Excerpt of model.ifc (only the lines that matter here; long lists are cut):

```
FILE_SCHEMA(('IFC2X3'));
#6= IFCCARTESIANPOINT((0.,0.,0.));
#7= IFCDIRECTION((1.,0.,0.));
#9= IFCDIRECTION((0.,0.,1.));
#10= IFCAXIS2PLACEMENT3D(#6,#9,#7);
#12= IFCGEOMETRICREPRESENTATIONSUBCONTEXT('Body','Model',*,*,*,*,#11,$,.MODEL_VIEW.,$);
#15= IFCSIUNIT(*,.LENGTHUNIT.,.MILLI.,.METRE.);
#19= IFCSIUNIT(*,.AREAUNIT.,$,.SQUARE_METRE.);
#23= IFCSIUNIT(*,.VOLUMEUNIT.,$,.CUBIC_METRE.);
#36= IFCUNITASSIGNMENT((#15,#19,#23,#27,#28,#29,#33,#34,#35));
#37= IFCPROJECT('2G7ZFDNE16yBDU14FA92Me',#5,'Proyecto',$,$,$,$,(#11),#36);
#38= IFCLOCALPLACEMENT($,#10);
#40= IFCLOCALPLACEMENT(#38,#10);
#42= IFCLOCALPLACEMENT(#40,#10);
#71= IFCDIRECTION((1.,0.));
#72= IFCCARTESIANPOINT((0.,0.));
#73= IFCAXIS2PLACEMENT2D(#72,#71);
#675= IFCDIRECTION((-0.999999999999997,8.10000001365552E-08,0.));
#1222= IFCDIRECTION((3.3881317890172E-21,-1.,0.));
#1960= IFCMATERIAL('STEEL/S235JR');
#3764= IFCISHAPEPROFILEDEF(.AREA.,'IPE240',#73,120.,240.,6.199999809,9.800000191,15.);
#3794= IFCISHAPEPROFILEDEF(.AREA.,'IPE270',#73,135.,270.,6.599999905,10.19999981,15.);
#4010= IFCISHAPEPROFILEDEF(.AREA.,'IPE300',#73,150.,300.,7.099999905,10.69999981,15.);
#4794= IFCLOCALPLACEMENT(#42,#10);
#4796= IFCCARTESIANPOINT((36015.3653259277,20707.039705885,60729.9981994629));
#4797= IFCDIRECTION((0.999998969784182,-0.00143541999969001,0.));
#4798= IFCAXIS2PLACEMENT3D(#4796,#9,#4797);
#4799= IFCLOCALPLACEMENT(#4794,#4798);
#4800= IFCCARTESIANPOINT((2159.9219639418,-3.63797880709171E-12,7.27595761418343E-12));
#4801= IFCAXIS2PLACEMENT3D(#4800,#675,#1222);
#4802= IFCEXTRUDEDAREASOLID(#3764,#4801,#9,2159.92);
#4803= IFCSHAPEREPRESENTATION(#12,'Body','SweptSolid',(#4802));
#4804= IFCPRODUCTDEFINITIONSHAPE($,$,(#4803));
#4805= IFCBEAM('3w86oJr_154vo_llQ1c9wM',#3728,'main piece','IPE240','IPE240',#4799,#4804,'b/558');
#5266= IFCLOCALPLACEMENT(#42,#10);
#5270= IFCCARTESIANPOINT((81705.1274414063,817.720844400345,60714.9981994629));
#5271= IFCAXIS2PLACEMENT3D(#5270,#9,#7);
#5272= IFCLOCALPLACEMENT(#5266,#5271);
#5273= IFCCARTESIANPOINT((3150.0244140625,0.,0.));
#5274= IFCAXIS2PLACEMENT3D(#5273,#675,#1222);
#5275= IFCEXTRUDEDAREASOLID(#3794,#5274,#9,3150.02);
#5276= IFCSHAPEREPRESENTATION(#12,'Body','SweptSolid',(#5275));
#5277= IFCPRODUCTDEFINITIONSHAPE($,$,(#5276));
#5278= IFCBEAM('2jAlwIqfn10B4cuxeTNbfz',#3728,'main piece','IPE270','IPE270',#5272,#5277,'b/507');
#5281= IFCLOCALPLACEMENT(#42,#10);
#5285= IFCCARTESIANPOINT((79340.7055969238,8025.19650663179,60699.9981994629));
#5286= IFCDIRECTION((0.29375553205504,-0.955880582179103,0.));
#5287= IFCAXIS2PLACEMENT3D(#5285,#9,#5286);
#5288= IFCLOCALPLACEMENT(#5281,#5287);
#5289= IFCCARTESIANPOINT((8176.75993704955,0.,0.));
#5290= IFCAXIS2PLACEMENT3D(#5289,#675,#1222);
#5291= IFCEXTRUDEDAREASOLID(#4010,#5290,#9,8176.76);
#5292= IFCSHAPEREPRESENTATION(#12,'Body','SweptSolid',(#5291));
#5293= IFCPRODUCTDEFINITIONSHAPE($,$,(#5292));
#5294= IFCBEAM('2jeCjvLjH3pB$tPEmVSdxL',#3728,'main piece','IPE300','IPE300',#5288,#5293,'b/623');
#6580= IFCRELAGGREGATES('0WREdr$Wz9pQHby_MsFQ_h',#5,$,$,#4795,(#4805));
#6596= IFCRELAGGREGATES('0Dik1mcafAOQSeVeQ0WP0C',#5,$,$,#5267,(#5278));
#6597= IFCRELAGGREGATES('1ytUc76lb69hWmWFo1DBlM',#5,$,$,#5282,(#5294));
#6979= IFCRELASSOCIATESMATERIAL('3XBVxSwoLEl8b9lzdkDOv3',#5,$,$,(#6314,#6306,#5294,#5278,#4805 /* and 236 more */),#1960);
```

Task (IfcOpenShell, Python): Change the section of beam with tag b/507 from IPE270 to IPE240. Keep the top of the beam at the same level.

```python
import ifcopenshell
import ifcopenshell.util.element
import ifcopenshell.util.representation

model = ifcopenshell.open("model.ifc")

member = model.by_guid("2jAlwIqfn10B4cuxeTNbfz")
source = next(p for p in model.by_type("IfcIShapeProfileDef") if p.ProfileName == "IPE240")

body = ifcopenshell.util.representation.get_representation(member, "Model", "Body")
solid = body.Items[0]
old_profile = solid.SweptArea

# Copy the section's sizes but keep this member's own profile position.
profile = ifcopenshell.util.element.copy(model, source)
# Profiles are centred, so shift by half the change in depth to hold the top.
shift = (old_profile.OverallDepth - profile.OverallDepth) / 2
x, y = old_profile.Position.Location.Coordinates
up = (0.0, 1.0)  # upwards, in the solid's own plane
location = model.createIfcCartesianPoint((x + up[0] * shift, y + up[1] * shift))
profile.Position = model.createIfcAxis2Placement2D(location, old_profile.Position.RefDirection)
solid.SweptArea = profile
if not model.get_total_inverses(old_profile):
    ifcopenshell.util.element.remove_deep2(model, old_profile)
member.Description = member.Description.replace("IPE270", "IPE240")
member.ObjectType = member.ObjectType.replace("IPE270", "IPE240")

print(solid.SweptArea)

model.write("model-out.ifc")
```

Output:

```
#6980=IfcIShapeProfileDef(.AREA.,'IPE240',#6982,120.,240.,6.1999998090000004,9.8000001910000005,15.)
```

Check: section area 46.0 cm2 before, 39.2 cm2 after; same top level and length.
